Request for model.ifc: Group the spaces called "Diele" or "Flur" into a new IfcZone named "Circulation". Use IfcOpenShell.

First a look at what the model holds.

```python
import ifcopenshell

model = ifcopenshell.open("model.ifc")
print(model.schema)
seen = {}
for space in model.by_type("IfcSpace"):
    seen[space.LongName] = seen.get(space.LongName, 0) + 1
for name, count in sorted(seen.items(), key=str):
    print(count, "x", name)
print("zones:", [z.Name for z in model.by_type("IfcZone")][:20])
```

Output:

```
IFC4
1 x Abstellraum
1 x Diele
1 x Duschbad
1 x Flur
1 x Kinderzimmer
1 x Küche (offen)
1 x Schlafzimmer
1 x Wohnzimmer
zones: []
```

```python
import ifcopenshell
import ifcopenshell.api.group
import ifcopenshell.api.root

model = ifcopenshell.open("model.ifc")

names = {"Diele", "Flur"}
spaces = [s for s in model.by_type("IfcSpace") if s.LongName in names]

zone = ifcopenshell.api.root.create_entity(model, ifc_class="IfcZone", name="Circulation")
ifcopenshell.api.group.assign_group(model, products=spaces, group=zone)
print(len(spaces), "spaces in", zone.Name)

model.write("model_rev.ifc")
```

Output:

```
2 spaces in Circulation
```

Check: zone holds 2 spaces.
